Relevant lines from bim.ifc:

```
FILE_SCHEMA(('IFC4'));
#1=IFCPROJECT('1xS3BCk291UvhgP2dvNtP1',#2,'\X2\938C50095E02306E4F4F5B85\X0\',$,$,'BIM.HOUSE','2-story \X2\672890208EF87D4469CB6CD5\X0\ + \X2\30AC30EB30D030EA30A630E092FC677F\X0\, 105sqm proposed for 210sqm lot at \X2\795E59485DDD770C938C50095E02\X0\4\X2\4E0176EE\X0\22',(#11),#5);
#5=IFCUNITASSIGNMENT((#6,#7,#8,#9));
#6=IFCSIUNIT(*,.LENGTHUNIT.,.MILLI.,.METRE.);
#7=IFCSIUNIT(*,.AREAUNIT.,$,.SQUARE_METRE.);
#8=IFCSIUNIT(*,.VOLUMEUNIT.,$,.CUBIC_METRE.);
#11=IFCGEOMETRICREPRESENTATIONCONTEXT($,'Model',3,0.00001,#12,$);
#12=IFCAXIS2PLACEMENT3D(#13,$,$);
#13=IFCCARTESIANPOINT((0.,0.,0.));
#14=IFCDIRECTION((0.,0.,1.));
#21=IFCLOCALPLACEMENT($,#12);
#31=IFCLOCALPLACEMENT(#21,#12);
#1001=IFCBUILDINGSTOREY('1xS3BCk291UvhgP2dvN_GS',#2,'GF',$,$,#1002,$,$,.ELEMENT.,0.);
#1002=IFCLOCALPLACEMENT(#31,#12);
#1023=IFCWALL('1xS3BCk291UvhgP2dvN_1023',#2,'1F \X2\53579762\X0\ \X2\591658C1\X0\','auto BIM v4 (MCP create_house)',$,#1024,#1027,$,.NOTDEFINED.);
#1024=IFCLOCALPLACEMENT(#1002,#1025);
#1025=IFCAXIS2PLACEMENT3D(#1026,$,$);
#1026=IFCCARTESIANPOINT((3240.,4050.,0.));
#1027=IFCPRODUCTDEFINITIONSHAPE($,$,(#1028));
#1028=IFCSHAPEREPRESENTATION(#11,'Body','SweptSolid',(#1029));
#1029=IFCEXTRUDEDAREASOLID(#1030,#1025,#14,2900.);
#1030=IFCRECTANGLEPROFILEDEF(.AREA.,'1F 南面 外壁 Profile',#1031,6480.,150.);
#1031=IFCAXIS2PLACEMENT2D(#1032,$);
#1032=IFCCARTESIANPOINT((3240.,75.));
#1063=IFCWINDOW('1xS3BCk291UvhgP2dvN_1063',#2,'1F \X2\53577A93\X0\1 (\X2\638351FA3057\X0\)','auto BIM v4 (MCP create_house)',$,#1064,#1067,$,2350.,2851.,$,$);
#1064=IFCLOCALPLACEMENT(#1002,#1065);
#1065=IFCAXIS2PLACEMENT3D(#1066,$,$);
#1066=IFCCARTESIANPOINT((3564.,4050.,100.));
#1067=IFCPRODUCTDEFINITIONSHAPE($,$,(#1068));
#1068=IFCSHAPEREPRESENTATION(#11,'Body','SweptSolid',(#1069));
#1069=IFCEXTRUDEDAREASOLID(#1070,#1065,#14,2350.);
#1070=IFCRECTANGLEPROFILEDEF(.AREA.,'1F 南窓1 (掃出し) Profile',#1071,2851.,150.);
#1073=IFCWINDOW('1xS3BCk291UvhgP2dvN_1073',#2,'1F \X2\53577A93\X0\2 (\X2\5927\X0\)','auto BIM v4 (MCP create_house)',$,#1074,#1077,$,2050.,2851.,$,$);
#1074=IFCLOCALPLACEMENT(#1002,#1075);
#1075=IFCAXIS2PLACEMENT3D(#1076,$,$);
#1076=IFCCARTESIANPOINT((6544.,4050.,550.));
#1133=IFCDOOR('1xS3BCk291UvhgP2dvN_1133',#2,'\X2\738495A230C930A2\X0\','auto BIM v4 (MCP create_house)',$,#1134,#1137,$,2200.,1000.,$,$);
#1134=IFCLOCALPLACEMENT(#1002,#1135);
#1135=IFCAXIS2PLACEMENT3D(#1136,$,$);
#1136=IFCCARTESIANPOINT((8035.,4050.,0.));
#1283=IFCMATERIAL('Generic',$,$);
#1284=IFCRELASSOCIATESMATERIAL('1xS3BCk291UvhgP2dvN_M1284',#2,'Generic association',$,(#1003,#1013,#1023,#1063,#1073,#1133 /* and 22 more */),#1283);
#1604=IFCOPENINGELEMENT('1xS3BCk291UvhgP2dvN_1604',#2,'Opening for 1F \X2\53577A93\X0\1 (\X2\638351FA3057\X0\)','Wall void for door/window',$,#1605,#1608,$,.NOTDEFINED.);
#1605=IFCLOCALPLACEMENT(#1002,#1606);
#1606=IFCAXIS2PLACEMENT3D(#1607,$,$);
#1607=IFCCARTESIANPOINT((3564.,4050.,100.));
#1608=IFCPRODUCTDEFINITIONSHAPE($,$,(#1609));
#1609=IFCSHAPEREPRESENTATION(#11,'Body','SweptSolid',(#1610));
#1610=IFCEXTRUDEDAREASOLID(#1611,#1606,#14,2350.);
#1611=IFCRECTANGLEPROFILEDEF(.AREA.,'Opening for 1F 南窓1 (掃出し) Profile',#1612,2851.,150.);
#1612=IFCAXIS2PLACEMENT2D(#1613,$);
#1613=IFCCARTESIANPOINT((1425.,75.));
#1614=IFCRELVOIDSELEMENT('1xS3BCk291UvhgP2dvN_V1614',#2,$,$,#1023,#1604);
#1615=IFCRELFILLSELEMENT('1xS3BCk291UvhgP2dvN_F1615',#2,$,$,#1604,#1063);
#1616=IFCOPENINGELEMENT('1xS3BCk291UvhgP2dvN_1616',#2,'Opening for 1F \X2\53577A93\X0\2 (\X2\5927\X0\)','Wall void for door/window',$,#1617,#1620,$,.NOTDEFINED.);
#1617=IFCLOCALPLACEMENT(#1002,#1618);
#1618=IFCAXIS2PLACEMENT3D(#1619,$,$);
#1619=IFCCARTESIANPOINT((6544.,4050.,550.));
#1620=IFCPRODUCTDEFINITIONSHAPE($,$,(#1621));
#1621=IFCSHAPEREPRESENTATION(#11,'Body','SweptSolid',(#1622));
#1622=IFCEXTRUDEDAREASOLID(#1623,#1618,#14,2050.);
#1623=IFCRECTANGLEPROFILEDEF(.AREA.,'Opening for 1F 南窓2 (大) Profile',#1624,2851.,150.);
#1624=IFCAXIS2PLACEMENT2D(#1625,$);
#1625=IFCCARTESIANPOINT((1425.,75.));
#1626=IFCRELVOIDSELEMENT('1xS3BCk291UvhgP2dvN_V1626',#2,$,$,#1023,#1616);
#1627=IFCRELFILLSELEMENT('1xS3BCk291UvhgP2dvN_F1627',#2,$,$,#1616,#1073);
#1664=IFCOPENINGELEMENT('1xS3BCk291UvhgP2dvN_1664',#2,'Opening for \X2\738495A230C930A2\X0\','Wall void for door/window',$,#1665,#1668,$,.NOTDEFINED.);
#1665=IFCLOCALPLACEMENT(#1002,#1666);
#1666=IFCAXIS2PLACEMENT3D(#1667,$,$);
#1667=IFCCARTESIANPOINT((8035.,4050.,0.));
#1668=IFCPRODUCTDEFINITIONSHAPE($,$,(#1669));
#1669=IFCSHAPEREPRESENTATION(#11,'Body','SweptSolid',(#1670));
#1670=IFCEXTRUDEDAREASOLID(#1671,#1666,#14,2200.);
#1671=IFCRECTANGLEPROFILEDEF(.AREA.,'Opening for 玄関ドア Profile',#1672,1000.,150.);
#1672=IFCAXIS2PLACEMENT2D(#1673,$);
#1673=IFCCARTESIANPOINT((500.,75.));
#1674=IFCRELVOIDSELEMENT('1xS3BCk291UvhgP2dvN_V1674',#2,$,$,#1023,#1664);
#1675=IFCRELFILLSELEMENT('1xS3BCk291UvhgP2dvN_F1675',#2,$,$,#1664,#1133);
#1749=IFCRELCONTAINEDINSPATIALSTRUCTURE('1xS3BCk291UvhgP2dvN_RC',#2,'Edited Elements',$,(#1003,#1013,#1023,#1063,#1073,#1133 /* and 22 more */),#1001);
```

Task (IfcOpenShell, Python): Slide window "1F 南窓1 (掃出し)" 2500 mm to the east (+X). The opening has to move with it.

```python
import ifcopenshell
import ifcopenshell.api.geometry
import ifcopenshell.util.placement
import ifcopenshell.util.unit

model = ifcopenshell.open("bim.ifc")
unit_scale = ifcopenshell.util.unit.calculate_unit_scale(model)

window = model.by_id(1063)
opening = window.FillsVoids[0].RelatingOpeningElement
wall = opening.VoidsElements[0].RelatingBuildingElement

wall_matrix = ifcopenshell.util.placement.get_local_placement(wall.ObjectPlacement)
shift = wall_matrix[:3, 0] * 2.5 / unit_scale
before = ifcopenshell.util.placement.get_local_placement(window.ObjectPlacement)[:3, 3].copy()

# The window is not placed relative to its opening, so move both.
for product in (opening, window):
    matrix = ifcopenshell.util.placement.get_local_placement(product.ObjectPlacement)
    matrix[:3, 3] += shift
    ifcopenshell.api.geometry.edit_object_placement(model, product=product, matrix=matrix, is_si=False)

after = ifcopenshell.util.placement.get_local_placement(window.ObjectPlacement)[:3, 3]
print("window moved by", (after - before).round(3) + 0.0)

model.write("bim-out.ifc")
```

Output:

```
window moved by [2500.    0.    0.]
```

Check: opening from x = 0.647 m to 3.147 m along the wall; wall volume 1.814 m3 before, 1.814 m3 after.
